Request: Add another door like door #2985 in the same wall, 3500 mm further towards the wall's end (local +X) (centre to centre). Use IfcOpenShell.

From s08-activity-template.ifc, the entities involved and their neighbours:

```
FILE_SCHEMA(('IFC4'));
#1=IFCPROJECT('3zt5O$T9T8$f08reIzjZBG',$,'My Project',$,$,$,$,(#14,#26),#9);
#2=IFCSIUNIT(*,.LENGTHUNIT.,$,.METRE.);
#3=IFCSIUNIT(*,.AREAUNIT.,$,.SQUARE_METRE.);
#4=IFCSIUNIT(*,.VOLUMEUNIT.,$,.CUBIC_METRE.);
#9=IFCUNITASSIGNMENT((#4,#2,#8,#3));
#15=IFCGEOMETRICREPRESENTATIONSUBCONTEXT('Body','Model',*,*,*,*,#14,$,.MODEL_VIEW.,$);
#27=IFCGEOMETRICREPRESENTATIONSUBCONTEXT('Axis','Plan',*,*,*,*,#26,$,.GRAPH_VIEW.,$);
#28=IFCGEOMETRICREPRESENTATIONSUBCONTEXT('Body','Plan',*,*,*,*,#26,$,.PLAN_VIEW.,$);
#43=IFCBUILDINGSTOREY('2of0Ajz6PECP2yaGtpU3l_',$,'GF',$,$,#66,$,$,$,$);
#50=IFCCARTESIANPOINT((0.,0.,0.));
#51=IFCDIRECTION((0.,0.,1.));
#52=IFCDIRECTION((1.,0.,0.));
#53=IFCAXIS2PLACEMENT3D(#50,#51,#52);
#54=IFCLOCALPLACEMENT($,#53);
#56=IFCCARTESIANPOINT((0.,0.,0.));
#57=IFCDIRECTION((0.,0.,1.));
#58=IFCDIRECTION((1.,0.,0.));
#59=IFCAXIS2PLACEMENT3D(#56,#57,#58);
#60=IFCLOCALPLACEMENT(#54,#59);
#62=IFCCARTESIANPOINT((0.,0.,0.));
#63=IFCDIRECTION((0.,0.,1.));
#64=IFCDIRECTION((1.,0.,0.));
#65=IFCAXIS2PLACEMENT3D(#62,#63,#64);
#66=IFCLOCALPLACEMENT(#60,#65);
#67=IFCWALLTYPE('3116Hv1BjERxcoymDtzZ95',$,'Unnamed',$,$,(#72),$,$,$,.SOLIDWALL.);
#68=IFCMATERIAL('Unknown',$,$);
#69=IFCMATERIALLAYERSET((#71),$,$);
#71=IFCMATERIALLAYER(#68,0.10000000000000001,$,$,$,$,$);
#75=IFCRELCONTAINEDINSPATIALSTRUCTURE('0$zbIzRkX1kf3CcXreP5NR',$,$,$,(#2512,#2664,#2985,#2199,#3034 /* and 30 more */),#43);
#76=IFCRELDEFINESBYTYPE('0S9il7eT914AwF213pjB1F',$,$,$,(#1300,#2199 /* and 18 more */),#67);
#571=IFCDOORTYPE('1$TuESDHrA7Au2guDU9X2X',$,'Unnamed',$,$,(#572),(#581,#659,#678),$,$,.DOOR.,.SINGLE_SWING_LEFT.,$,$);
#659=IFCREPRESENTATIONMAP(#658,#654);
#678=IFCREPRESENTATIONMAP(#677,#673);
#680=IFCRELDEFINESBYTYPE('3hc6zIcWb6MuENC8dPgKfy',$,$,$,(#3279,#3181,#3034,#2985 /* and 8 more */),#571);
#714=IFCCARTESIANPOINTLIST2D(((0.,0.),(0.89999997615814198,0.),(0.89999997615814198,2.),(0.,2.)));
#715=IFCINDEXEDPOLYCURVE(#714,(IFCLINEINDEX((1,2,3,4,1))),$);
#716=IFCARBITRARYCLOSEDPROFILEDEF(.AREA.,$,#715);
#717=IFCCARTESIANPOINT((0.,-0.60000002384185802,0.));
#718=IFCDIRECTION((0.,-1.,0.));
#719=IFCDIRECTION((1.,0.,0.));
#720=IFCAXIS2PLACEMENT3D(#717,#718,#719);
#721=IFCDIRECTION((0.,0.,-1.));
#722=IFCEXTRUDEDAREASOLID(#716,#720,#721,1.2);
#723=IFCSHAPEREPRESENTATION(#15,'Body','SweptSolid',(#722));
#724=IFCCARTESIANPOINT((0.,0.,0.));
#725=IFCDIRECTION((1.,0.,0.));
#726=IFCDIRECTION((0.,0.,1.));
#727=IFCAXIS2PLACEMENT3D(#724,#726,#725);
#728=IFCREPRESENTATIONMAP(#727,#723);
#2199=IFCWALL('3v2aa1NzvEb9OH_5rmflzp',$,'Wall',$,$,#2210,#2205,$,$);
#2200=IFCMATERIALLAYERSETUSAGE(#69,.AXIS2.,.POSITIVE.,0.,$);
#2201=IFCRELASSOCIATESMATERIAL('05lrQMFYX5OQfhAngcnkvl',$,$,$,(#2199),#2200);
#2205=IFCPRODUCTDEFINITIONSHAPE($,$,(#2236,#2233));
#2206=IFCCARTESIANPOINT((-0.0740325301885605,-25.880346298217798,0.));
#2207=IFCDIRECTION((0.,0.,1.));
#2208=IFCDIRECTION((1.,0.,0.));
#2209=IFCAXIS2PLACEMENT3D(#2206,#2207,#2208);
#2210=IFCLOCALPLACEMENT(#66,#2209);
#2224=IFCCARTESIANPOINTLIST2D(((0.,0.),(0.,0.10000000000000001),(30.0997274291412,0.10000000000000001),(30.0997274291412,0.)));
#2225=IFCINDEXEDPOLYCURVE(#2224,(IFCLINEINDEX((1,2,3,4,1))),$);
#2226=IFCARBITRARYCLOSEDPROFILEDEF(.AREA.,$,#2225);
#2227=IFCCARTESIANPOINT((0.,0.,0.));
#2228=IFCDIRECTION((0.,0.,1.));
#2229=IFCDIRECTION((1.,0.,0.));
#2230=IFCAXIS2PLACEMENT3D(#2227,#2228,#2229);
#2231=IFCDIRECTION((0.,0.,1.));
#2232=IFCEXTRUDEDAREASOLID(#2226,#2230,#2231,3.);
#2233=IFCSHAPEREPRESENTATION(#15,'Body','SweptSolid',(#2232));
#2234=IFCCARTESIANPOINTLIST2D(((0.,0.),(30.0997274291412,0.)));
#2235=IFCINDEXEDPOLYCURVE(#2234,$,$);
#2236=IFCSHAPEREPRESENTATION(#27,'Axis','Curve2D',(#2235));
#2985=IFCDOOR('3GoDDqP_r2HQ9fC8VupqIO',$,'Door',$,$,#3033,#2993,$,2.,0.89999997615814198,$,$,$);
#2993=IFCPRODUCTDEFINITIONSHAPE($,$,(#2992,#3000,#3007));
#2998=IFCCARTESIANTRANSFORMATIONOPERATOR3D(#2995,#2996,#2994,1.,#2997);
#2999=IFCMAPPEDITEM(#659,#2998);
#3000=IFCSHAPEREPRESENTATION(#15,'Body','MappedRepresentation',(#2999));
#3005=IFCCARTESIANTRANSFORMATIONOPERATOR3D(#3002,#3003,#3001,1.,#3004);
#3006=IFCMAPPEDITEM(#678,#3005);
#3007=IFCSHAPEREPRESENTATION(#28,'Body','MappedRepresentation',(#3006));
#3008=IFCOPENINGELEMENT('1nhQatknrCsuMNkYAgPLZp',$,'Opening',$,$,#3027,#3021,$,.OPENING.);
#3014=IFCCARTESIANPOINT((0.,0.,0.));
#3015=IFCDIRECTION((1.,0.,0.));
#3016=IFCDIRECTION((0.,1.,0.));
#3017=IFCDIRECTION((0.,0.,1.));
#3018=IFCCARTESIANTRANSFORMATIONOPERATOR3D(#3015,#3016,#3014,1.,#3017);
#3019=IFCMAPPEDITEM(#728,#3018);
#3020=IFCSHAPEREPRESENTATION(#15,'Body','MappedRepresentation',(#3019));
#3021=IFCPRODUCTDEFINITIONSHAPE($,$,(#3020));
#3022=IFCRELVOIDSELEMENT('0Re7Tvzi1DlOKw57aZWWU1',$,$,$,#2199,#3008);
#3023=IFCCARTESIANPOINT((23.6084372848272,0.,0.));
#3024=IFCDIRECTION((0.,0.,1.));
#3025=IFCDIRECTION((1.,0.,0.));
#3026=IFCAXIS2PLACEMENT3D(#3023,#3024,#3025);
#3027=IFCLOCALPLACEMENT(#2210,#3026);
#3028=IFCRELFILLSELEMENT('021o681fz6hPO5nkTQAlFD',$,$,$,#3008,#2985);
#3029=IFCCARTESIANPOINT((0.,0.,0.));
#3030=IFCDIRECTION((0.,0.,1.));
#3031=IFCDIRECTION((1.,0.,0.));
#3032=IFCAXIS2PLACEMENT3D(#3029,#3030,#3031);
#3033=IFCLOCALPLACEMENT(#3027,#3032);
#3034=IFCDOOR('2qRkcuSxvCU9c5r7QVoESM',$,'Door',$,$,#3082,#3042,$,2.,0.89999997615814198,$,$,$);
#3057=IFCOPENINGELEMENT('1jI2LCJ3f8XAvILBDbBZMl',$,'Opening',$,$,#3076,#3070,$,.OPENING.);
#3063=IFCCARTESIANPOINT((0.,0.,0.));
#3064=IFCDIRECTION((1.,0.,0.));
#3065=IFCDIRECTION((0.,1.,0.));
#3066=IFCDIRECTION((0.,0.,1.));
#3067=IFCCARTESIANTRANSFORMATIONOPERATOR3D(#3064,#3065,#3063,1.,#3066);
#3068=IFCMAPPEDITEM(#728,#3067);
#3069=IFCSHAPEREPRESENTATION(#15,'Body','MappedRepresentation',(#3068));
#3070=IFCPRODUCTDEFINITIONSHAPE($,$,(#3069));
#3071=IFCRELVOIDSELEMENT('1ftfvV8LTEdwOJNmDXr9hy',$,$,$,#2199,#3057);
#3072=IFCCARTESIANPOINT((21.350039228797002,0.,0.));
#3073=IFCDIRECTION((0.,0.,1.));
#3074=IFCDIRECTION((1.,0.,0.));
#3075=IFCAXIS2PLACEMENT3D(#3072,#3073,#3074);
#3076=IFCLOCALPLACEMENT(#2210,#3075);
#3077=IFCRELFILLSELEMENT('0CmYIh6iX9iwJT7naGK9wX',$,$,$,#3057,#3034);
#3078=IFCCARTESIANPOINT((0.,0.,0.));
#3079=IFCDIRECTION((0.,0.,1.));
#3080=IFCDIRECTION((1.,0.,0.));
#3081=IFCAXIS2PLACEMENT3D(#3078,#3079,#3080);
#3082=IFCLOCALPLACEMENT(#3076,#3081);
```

```python
import ifcopenshell
import ifcopenshell.api.feature
import ifcopenshell.api.geometry
import ifcopenshell.api.root
import ifcopenshell.geom
import ifcopenshell.util.element
import ifcopenshell.util.placement
import ifcopenshell.util.shape
import ifcopenshell.util.unit

model = ifcopenshell.open("s08-activity-template.ifc")
unit_scale = ifcopenshell.util.unit.calculate_unit_scale(model)
settings = ifcopenshell.geom.settings()


def volume(element):
    """Net volume in cubic metres, openings subtracted."""
    shape = ifcopenshell.geom.create_shape(settings, element)
    return ifcopenshell.util.shape.get_volume(shape.geometry)


door = model.by_guid("3GoDDqP_r2HQ9fC8VupqIO")
opening = door.FillsVoids[0].RelatingOpeningElement
wall = opening.VoidsElements[0].RelatingBuildingElement
before = volume(wall)
shift = ifcopenshell.util.placement.get_local_placement(wall.ObjectPlacement)[:3, 0] * 3.5 / unit_scale

# copy_class copies the void relationship, type, container and properties, but no geometry.
new_opening = ifcopenshell.api.root.copy_class(model, product=opening)
new_opening.Representation = ifcopenshell.util.element.copy_deep(
    model, opening.Representation, exclude=["IfcGeometricRepresentationContext", "IfcRepresentationMap"]
)
new_door = ifcopenshell.api.root.copy_class(model, product=door)
new_door.Representation = ifcopenshell.util.element.copy_deep(
    model, door.Representation, exclude=["IfcGeometricRepresentationContext", "IfcRepresentationMap"]
)
ifcopenshell.api.feature.add_filling(model, opening=new_opening, element=new_door)

for old, new in ((opening, new_opening), (door, new_door)):
    matrix = ifcopenshell.util.placement.get_local_placement(old.ObjectPlacement)
    matrix[:3, 3] += shift
    ifcopenshell.api.geometry.edit_object_placement(model, product=new, matrix=matrix, is_si=False)

after = volume(wall)

print(f"wall volume {before:.3f} -> {after:.3f} m3")

model.write("s08-activity-template_v2.ifc")
```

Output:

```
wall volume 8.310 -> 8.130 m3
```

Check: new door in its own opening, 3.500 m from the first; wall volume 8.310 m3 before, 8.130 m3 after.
